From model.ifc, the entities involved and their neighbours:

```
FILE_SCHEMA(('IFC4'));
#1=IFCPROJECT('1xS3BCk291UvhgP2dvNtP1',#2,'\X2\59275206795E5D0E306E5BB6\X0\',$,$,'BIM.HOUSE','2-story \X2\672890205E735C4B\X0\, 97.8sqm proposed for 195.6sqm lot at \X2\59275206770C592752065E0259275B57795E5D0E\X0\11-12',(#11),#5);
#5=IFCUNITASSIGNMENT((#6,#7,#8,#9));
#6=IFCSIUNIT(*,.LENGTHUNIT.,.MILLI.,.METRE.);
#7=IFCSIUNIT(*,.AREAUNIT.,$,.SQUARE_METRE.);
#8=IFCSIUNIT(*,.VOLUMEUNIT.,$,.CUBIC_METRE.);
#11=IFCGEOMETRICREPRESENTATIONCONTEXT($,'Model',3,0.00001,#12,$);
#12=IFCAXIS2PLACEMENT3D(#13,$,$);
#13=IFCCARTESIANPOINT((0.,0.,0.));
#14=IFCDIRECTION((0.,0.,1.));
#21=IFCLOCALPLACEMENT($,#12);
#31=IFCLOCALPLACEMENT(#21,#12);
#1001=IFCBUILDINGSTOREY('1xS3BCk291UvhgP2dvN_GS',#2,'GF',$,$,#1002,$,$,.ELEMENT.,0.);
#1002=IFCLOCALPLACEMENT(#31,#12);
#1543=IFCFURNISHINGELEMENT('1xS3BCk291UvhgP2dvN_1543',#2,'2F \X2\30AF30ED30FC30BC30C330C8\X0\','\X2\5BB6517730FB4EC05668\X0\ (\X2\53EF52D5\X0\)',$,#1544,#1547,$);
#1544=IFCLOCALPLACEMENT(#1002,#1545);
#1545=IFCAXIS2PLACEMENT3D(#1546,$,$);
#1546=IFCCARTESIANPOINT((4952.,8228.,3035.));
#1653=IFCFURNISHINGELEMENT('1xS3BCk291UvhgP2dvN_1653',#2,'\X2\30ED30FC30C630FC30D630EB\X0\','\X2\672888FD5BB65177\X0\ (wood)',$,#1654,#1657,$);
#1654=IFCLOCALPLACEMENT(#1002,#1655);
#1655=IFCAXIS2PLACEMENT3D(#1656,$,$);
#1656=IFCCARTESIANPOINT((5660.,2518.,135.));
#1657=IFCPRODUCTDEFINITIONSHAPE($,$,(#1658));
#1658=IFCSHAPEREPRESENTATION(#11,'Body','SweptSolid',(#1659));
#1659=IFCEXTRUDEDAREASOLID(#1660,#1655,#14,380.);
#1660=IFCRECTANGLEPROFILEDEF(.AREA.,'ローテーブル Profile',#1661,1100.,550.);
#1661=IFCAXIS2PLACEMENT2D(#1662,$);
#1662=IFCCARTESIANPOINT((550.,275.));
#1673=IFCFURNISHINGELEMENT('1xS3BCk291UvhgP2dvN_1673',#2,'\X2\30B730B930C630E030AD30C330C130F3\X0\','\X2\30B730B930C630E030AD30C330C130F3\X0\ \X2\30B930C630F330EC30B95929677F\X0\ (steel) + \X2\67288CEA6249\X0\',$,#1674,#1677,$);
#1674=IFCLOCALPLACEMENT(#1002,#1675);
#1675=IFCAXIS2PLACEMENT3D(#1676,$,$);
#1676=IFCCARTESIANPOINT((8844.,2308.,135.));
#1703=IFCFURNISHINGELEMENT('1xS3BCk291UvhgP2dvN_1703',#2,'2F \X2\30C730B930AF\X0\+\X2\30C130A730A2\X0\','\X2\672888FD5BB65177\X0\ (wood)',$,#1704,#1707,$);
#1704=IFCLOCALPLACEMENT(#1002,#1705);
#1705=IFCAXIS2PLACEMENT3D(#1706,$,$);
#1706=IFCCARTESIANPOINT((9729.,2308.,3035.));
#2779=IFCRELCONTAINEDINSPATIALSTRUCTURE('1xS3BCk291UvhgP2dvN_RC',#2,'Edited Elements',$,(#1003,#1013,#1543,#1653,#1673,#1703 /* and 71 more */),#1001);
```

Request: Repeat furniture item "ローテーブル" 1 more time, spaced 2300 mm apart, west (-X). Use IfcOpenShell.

```python
import numpy as np
import ifcopenshell
import ifcopenshell.api.geometry
import ifcopenshell.api.root
import ifcopenshell.util.element
import ifcopenshell.util.placement

model = ifcopenshell.open("model.ifc")


def reuse_history(source, copy):
    """copy_class also copies each property set's owner history, people and application; keep the originals."""
    for rel in copy.IsDefinedBy:
        if rel.is_a("IfcRelDefinesByProperties") and (history := rel.RelatingPropertyDefinition.OwnerHistory):
            rel.RelatingPropertyDefinition.OwnerHistory = source.OwnerHistory
            ifcopenshell.util.element.remove_deep2(model, history)


source = model.by_guid("1xS3BCk291UvhgP2dvN_1653")
base = ifcopenshell.util.placement.get_local_placement(source.ObjectPlacement)
step = np.array([-1.0, 0.0, 0.0]) * 2300.0

for i in range(1, 2):
    copy = ifcopenshell.api.root.copy_class(model, product=source)
    copy.Representation = ifcopenshell.util.element.copy_deep(
        model, source.Representation, exclude=["IfcGeometricRepresentationContext", "IfcRepresentationMap"]
    )
    reuse_history(source, copy)
    matrix = base.copy()
    matrix[:3, 3] += i * step
    print("added at", matrix[:3, 3].round(3) + 0.0)
    ifcopenshell.api.geometry.edit_object_placement(model, product=copy, matrix=matrix, is_si=False)

model.write("model_v2.ifc")
```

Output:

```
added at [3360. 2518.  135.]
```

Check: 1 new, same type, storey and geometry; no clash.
